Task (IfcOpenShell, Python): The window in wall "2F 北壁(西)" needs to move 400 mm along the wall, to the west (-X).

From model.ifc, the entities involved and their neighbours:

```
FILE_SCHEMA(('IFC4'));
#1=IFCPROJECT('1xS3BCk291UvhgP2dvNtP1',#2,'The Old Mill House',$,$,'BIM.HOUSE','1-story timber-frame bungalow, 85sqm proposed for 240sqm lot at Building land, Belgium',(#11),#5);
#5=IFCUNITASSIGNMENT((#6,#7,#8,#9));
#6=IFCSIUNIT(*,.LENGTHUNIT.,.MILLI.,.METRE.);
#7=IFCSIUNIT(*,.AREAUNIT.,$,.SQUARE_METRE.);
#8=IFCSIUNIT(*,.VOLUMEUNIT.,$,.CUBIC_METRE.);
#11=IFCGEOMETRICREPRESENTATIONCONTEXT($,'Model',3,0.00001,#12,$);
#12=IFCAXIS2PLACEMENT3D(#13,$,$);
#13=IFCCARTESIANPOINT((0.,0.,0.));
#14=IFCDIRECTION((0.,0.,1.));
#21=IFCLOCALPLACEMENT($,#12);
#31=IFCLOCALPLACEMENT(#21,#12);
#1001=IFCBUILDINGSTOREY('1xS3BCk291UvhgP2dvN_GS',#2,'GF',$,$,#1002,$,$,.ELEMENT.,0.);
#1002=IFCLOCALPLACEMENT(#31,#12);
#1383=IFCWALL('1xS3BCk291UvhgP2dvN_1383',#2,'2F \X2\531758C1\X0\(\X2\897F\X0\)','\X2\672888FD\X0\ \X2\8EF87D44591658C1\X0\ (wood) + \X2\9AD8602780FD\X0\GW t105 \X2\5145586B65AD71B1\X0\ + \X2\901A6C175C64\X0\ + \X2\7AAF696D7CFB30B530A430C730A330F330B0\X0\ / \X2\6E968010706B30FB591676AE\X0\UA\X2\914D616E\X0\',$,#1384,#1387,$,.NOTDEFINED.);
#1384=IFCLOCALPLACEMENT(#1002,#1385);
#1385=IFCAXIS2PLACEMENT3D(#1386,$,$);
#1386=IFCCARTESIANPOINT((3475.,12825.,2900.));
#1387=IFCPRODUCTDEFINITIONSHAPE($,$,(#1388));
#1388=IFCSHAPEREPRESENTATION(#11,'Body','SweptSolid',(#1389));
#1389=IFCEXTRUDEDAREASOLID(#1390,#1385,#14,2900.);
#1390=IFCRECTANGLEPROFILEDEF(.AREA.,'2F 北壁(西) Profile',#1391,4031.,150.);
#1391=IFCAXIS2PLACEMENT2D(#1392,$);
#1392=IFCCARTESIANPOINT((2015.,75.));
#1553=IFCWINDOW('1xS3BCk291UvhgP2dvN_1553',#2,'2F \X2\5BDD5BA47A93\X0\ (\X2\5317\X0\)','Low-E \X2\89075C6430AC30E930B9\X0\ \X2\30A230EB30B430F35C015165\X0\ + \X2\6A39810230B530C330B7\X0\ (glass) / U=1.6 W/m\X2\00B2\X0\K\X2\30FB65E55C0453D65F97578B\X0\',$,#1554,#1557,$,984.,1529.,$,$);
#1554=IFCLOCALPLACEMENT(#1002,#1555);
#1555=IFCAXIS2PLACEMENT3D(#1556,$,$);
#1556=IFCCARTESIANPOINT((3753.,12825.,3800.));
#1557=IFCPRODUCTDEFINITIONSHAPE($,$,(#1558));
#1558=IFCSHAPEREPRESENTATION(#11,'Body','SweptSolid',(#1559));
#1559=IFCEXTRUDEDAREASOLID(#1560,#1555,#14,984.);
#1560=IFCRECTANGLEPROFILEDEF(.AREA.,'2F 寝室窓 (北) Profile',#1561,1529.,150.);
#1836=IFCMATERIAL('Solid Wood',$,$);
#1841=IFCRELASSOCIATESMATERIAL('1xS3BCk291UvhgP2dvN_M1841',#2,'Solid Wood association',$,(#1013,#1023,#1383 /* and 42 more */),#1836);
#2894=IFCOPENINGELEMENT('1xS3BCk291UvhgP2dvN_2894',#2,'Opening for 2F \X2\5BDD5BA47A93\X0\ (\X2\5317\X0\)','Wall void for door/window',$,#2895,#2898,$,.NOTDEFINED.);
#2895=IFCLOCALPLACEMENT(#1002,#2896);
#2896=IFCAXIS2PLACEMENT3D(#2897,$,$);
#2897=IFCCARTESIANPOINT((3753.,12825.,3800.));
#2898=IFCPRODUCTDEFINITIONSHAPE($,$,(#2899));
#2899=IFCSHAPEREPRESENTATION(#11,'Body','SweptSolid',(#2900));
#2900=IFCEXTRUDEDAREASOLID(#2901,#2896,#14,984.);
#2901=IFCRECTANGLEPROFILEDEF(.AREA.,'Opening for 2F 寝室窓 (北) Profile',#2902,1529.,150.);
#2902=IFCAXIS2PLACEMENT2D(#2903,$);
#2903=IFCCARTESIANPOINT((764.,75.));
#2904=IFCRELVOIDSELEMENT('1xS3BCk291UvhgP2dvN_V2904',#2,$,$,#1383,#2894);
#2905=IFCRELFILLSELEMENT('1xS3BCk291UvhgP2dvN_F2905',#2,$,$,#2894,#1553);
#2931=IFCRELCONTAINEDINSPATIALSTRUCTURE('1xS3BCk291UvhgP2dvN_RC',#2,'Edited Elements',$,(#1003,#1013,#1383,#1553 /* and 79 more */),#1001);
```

```python
import ifcopenshell
import ifcopenshell.api.geometry
import ifcopenshell.util.placement
import ifcopenshell.util.unit

model = ifcopenshell.open("model.ifc")
unit_scale = ifcopenshell.util.unit.calculate_unit_scale(model)

window = model.by_id(1553)
opening = window.FillsVoids[0].RelatingOpeningElement
wall = opening.VoidsElements[0].RelatingBuildingElement

wall_matrix = ifcopenshell.util.placement.get_local_placement(wall.ObjectPlacement)
shift = wall_matrix[:3, 0] * -0.4 / unit_scale
before = ifcopenshell.util.placement.get_local_placement(window.ObjectPlacement)[:3, 3].copy()

# The window is not placed relative to its opening, so move both.
for product in (opening, window):
    matrix = ifcopenshell.util.placement.get_local_placement(product.ObjectPlacement)
    matrix[:3, 3] += shift
    ifcopenshell.api.geometry.edit_object_placement(model, product=product, matrix=matrix, is_si=False)

after = ifcopenshell.util.placement.get_local_placement(window.ObjectPlacement)[:3, 3]
print("window moved by", (after - before).round(3) + 0.0)

model.write("model_v2.ifc")
```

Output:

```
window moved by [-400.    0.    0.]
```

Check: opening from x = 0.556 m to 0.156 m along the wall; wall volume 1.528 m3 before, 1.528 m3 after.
